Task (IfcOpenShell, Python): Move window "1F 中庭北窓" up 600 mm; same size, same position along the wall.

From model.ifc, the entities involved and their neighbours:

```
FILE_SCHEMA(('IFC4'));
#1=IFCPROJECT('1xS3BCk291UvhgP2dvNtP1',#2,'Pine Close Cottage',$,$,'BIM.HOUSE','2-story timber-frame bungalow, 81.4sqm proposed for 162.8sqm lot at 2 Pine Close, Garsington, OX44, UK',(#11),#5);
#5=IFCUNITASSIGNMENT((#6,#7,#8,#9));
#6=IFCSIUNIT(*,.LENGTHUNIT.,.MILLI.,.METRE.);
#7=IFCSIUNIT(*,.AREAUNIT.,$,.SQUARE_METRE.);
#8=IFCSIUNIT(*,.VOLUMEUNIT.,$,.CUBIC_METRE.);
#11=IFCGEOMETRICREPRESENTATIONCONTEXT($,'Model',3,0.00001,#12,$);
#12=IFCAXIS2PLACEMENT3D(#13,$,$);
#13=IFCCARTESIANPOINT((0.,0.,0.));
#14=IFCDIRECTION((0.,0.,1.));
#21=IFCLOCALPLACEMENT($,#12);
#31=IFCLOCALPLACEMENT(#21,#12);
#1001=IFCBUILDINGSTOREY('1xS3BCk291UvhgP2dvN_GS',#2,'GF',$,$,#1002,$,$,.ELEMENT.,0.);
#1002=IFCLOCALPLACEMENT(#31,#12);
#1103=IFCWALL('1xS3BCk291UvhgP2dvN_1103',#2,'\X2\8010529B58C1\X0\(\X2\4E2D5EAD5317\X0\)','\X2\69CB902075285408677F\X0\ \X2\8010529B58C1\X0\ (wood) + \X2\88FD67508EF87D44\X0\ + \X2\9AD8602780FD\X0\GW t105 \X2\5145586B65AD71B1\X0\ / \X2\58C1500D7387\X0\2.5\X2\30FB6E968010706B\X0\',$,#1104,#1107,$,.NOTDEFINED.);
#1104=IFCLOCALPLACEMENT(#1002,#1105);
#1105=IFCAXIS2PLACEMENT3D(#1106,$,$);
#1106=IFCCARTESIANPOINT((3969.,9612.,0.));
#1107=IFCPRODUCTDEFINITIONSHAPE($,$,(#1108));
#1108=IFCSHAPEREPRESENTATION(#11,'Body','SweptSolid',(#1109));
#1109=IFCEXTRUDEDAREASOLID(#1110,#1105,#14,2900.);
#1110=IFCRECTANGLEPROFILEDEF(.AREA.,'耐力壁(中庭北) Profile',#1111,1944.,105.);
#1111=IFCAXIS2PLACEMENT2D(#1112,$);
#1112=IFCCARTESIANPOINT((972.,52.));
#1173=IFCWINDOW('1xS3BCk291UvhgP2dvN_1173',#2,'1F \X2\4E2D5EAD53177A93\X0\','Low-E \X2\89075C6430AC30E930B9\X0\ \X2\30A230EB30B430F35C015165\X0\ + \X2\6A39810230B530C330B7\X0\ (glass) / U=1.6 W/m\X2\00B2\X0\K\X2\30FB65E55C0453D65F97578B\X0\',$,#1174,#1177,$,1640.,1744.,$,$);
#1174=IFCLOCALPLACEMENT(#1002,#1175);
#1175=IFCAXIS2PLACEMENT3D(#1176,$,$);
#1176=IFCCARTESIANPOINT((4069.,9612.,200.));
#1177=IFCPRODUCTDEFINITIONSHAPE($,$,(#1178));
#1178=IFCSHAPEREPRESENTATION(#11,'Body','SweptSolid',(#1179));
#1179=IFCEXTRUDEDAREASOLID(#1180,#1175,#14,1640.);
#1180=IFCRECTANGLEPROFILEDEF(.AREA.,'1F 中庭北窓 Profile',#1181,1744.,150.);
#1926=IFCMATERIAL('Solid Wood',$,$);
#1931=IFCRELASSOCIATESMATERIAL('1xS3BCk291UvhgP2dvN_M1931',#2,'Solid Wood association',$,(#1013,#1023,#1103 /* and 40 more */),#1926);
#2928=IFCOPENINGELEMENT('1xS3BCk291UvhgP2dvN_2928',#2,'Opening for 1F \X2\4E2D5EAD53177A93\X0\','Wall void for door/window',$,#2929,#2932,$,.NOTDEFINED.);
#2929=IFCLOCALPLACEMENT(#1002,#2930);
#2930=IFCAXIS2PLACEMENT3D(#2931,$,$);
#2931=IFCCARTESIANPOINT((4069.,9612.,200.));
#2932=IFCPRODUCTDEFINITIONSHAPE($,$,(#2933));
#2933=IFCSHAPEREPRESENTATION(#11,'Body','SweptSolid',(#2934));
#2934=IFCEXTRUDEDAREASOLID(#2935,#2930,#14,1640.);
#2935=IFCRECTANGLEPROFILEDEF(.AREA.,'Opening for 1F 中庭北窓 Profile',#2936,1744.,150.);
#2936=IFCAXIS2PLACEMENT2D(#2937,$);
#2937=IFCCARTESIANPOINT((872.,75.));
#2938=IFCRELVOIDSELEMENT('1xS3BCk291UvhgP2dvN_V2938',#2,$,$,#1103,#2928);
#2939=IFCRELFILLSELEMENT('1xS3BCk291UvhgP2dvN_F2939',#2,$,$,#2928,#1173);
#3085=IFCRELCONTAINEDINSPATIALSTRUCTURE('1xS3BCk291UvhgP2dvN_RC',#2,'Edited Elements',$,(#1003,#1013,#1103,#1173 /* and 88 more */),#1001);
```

```python
import numpy as np
import ifcopenshell
import ifcopenshell.api.geometry
import ifcopenshell.util.placement
import ifcopenshell.util.unit

model = ifcopenshell.open("model.ifc")
unit_scale = ifcopenshell.util.unit.calculate_unit_scale(model)

window = model.by_guid("1xS3BCk291UvhgP2dvN_1173")
opening = window.FillsVoids[0].RelatingOpeningElement
dz = 0.6 / unit_scale

shift = np.array([0.0, 0.0, dz])
# The window is not placed relative to its opening, so move both.
for product in (opening, window):
    matrix = ifcopenshell.util.placement.get_local_placement(product.ObjectPlacement)
    matrix[:3, 3] += shift
    ifcopenshell.api.geometry.edit_object_placement(model, product=product, matrix=matrix, is_si=False)

print(f"moved by {dz * unit_scale:+.3f} m")

model.write("model-out.ifc")
```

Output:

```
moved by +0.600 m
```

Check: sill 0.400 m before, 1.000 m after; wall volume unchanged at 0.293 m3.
